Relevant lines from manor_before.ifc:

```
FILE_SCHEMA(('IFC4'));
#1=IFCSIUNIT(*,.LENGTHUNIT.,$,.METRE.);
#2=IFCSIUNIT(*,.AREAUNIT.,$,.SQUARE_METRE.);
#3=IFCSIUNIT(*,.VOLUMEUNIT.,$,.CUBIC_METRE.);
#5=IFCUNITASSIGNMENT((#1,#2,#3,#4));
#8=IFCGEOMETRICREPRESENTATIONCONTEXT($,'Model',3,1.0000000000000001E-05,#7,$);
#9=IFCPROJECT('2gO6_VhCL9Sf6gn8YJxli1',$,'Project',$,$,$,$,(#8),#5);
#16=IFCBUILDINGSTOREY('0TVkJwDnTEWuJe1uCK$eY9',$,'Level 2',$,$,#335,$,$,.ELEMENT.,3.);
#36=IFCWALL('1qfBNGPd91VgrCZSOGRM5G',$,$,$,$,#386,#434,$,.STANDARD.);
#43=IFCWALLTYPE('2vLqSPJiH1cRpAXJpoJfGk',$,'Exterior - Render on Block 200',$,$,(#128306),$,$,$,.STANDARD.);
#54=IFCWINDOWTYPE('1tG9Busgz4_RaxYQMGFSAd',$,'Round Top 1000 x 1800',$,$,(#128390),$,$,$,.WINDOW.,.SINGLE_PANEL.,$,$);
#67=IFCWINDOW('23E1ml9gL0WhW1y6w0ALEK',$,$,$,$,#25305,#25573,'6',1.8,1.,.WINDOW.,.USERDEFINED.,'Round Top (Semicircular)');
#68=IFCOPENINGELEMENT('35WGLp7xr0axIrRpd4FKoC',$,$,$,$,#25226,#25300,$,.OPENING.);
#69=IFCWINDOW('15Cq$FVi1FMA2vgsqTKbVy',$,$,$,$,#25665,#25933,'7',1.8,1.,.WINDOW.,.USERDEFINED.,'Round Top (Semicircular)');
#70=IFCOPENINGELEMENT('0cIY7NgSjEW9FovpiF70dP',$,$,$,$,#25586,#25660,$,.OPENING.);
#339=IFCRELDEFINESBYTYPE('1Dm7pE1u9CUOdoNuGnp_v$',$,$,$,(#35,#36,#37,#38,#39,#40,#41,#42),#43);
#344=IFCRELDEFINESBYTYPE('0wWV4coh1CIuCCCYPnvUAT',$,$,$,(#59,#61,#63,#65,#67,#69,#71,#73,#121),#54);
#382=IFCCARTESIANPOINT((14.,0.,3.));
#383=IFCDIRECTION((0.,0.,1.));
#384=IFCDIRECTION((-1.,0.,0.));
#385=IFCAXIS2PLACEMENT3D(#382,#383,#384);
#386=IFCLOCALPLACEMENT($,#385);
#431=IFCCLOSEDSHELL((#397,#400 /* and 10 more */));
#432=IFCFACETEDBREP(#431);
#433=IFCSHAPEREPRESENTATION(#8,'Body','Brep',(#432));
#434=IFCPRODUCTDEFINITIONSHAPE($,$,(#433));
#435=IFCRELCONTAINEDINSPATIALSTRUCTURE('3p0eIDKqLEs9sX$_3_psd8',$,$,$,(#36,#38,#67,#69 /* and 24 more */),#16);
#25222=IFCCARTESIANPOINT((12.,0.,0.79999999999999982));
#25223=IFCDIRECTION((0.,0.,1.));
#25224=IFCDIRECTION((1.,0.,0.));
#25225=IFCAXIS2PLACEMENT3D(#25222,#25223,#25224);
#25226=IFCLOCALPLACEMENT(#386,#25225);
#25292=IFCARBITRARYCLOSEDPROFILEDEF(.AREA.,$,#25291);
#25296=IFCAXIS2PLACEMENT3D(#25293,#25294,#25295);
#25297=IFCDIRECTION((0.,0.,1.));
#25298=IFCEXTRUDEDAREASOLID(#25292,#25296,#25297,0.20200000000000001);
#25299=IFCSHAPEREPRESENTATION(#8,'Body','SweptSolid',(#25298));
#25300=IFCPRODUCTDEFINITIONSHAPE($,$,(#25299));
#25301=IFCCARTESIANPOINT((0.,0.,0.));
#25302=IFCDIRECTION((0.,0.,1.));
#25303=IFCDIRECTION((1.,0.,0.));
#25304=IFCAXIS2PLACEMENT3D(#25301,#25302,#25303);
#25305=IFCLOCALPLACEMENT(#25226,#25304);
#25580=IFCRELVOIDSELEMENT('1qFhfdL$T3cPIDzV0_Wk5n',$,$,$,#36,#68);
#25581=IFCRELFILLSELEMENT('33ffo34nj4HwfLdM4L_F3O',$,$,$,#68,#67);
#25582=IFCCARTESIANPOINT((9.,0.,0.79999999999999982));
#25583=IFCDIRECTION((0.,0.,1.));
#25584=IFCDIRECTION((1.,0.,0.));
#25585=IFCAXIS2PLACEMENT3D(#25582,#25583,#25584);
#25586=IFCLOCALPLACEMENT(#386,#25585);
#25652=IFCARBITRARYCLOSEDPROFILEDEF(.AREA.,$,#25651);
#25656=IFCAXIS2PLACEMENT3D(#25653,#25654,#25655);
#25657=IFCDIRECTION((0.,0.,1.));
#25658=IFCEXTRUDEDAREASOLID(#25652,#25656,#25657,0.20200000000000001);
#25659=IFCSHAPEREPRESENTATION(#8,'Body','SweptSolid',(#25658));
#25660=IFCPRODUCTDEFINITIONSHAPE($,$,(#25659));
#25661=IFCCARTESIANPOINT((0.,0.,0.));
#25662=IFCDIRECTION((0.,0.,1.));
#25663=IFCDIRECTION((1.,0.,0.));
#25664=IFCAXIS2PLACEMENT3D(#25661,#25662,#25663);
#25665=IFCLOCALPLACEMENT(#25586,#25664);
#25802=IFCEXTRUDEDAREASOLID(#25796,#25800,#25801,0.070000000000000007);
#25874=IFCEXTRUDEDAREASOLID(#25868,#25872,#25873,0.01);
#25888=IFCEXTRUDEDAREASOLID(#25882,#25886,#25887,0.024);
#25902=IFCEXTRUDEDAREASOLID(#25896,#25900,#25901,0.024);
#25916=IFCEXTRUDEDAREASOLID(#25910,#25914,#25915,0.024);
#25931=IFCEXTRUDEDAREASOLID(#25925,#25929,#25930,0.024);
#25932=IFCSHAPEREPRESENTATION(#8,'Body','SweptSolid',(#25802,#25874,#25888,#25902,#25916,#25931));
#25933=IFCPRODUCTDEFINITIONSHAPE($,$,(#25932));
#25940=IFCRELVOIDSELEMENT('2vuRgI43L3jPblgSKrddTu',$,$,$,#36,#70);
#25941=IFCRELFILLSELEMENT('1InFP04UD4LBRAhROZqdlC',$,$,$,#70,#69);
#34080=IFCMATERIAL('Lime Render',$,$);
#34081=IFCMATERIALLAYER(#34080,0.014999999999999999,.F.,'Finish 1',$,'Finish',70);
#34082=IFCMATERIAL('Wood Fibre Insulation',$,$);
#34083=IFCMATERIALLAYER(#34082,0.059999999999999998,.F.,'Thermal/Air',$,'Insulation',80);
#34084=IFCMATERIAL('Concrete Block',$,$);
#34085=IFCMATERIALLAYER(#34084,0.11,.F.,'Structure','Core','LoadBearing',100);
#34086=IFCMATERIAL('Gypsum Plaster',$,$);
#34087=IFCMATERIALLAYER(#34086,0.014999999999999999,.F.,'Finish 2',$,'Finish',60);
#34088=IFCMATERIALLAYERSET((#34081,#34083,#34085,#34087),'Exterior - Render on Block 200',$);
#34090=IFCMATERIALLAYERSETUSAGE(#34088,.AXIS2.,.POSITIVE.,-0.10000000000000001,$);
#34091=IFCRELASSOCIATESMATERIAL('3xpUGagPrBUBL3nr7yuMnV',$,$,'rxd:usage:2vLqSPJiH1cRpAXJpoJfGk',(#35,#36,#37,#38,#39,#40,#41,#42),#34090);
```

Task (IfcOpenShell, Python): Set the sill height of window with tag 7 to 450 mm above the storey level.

```python
import numpy as np
import ifcopenshell
import ifcopenshell.api.geometry
import ifcopenshell.geom
import ifcopenshell.util.element
import ifcopenshell.util.placement
import ifcopenshell.util.shape
import ifcopenshell.util.unit

model = ifcopenshell.open("manor_before.ifc")
unit_scale = ifcopenshell.util.unit.calculate_unit_scale(model)

window = model.by_id(69)
opening = window.FillsVoids[0].RelatingOpeningElement
storey = ifcopenshell.util.element.get_container(window, ifc_class="IfcBuildingStorey")
level = ifcopenshell.util.placement.get_local_placement(storey.ObjectPlacement)[2, 3]

# The opening's origin need not be at the sill, so measure its lowest point.
shape = ifcopenshell.geom.create_shape(ifcopenshell.geom.settings(), opening)
bottom = ifcopenshell.util.shape.get_shape_bottom_elevation(shape, shape.geometry) / unit_scale
dz = level + 0.45 - bottom

shift = np.array([0.0, 0.0, dz])
# The window is placed relative to its opening, so it follows when the opening moves.
matrix = ifcopenshell.util.placement.get_local_placement(opening.ObjectPlacement)
matrix[:3, 3] += shift
ifcopenshell.api.geometry.edit_object_placement(
    model, product=opening, matrix=matrix, is_si=False, should_transform_children=True
)

print(f"moved by {dz * unit_scale:+.3f} m")

model.write("manor_before_edited.ifc")
```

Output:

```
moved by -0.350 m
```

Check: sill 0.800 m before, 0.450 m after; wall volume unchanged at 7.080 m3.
